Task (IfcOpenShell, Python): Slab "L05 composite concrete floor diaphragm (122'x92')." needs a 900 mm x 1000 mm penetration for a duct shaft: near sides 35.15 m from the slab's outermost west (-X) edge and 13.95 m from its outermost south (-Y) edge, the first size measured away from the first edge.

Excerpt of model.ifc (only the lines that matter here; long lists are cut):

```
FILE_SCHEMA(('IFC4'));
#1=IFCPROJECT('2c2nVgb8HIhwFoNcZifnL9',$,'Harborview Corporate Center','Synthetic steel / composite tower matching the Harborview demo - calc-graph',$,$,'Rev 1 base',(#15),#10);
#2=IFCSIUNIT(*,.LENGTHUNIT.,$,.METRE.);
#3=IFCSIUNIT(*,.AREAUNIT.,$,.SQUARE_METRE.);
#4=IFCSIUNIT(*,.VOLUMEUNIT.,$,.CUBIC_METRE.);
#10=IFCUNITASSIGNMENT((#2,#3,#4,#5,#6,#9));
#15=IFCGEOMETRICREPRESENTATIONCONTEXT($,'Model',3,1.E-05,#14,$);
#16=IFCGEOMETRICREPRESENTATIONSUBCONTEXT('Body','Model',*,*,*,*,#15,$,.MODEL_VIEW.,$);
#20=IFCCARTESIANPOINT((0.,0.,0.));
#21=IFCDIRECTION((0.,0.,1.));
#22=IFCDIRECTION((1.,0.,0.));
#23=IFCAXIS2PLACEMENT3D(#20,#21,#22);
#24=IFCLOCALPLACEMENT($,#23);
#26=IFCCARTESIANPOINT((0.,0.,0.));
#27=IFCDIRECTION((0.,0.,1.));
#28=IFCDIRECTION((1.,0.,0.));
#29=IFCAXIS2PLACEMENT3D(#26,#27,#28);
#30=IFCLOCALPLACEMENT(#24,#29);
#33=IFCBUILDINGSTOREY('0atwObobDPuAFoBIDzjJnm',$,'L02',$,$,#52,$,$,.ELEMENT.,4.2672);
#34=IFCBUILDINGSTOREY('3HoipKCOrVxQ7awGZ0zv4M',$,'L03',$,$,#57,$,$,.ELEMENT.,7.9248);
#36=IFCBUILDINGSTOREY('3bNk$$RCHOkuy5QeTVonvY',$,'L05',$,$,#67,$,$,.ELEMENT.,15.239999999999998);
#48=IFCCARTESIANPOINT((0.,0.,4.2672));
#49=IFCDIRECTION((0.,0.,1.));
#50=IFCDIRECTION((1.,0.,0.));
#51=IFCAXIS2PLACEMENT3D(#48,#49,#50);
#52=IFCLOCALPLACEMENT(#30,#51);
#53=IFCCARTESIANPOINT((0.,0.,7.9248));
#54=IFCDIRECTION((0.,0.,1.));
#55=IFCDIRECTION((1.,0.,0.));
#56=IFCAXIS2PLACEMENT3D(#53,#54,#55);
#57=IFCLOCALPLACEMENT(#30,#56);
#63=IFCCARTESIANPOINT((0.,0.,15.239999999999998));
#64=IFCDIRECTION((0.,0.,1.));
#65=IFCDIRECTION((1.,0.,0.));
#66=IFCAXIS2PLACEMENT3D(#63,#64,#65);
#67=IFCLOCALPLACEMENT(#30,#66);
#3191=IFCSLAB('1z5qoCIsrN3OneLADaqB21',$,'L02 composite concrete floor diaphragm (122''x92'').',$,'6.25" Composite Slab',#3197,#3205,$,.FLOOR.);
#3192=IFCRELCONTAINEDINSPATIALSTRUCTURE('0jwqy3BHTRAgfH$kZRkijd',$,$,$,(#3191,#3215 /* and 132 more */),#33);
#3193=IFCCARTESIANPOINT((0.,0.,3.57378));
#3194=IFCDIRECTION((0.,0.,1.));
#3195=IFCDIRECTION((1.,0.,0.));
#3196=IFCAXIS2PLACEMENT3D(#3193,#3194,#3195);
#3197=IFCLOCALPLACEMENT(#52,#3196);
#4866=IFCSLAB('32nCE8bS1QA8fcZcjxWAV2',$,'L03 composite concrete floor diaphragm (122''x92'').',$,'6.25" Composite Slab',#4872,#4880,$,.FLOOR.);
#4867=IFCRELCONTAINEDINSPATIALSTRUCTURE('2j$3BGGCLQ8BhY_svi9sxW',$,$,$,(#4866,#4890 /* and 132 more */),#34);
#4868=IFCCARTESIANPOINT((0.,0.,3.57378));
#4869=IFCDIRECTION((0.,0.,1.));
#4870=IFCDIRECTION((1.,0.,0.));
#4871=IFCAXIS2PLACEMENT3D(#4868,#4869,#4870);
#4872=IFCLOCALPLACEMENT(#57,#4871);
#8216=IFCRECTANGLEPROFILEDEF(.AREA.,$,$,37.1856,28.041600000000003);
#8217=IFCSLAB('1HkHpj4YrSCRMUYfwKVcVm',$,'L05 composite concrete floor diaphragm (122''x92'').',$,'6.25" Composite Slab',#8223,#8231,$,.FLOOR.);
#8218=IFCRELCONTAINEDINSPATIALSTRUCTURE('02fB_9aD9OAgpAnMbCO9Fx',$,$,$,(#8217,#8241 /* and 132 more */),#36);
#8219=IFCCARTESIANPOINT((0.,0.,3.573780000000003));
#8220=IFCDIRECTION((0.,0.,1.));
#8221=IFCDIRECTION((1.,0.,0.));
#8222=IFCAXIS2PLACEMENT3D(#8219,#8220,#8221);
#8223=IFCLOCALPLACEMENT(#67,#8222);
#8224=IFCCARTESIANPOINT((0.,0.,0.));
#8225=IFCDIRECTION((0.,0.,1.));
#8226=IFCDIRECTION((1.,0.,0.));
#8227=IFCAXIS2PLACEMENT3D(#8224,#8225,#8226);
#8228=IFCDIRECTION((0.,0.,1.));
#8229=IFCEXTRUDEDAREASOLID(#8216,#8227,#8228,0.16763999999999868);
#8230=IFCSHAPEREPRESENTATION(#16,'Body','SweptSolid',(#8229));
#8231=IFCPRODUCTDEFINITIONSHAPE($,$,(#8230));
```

```python
import numpy as np
import ifcopenshell
import ifcopenshell.api.feature
import ifcopenshell.api.geometry
import ifcopenshell.api.root
import ifcopenshell.geom
import ifcopenshell.util.placement
import ifcopenshell.util.representation
import ifcopenshell.util.shape
import ifcopenshell.util.unit

model = ifcopenshell.open("model.ifc")
unit_scale = ifcopenshell.util.unit.calculate_unit_scale(model)
settings = ifcopenshell.geom.settings()


def volume(element):
    """Net volume in cubic metres, openings subtracted."""
    shape = ifcopenshell.geom.create_shape(settings, element)
    return ifcopenshell.util.shape.get_volume(shape.geometry)


slab = model.by_id(8217)
before = volume(slab)

# Extent in the slab's own axes, in metres. The edges named are its -X and -Y sides.
slab_shape = ifcopenshell.geom.create_shape(settings, slab)
vertices = ifcopenshell.util.shape.get_vertices(slab_shape.geometry)
x_min, y_min, bottom = vertices.min(axis=0)
top = vertices[:, 2].max()

opening = ifcopenshell.api.root.create_entity(model, ifc_class="IfcOpeningElement", name="Duct shaft opening", predefined_type="OPENING")
context = ifcopenshell.util.representation.get_context(model, "Model", "Body", "MODEL_VIEW")
width, depth = 0.9, 1
outline = [(0.0, 0.0), (width, 0.0), (width, depth), (0.0, depth), (0.0, 0.0)]
# Overshoot both faces by 50 mm so the cut is clean.
shape = ifcopenshell.api.geometry.add_slab_representation(
    model, context=context, depth=top - bottom + 0.1, polyline=outline
)
ifcopenshell.api.geometry.assign_representation(model, product=opening, representation=shape)

matrix = ifcopenshell.util.placement.get_local_placement(slab.ObjectPlacement)
matrix[:, 3] = matrix @ np.append(np.array([x_min + 35.15, y_min + 13.95, bottom - 0.05]) / unit_scale, 1.0)
ifcopenshell.api.geometry.edit_object_placement(model, product=opening, matrix=matrix, is_si=False)
ifcopenshell.api.feature.add_feature(model, feature=opening, element=slab)

after = volume(slab)

print(f"slab volume {before:.3f} -> {after:.3f} m3")

model.write("model_v2.ifc")
```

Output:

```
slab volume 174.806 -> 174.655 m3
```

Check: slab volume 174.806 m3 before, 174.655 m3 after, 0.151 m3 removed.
